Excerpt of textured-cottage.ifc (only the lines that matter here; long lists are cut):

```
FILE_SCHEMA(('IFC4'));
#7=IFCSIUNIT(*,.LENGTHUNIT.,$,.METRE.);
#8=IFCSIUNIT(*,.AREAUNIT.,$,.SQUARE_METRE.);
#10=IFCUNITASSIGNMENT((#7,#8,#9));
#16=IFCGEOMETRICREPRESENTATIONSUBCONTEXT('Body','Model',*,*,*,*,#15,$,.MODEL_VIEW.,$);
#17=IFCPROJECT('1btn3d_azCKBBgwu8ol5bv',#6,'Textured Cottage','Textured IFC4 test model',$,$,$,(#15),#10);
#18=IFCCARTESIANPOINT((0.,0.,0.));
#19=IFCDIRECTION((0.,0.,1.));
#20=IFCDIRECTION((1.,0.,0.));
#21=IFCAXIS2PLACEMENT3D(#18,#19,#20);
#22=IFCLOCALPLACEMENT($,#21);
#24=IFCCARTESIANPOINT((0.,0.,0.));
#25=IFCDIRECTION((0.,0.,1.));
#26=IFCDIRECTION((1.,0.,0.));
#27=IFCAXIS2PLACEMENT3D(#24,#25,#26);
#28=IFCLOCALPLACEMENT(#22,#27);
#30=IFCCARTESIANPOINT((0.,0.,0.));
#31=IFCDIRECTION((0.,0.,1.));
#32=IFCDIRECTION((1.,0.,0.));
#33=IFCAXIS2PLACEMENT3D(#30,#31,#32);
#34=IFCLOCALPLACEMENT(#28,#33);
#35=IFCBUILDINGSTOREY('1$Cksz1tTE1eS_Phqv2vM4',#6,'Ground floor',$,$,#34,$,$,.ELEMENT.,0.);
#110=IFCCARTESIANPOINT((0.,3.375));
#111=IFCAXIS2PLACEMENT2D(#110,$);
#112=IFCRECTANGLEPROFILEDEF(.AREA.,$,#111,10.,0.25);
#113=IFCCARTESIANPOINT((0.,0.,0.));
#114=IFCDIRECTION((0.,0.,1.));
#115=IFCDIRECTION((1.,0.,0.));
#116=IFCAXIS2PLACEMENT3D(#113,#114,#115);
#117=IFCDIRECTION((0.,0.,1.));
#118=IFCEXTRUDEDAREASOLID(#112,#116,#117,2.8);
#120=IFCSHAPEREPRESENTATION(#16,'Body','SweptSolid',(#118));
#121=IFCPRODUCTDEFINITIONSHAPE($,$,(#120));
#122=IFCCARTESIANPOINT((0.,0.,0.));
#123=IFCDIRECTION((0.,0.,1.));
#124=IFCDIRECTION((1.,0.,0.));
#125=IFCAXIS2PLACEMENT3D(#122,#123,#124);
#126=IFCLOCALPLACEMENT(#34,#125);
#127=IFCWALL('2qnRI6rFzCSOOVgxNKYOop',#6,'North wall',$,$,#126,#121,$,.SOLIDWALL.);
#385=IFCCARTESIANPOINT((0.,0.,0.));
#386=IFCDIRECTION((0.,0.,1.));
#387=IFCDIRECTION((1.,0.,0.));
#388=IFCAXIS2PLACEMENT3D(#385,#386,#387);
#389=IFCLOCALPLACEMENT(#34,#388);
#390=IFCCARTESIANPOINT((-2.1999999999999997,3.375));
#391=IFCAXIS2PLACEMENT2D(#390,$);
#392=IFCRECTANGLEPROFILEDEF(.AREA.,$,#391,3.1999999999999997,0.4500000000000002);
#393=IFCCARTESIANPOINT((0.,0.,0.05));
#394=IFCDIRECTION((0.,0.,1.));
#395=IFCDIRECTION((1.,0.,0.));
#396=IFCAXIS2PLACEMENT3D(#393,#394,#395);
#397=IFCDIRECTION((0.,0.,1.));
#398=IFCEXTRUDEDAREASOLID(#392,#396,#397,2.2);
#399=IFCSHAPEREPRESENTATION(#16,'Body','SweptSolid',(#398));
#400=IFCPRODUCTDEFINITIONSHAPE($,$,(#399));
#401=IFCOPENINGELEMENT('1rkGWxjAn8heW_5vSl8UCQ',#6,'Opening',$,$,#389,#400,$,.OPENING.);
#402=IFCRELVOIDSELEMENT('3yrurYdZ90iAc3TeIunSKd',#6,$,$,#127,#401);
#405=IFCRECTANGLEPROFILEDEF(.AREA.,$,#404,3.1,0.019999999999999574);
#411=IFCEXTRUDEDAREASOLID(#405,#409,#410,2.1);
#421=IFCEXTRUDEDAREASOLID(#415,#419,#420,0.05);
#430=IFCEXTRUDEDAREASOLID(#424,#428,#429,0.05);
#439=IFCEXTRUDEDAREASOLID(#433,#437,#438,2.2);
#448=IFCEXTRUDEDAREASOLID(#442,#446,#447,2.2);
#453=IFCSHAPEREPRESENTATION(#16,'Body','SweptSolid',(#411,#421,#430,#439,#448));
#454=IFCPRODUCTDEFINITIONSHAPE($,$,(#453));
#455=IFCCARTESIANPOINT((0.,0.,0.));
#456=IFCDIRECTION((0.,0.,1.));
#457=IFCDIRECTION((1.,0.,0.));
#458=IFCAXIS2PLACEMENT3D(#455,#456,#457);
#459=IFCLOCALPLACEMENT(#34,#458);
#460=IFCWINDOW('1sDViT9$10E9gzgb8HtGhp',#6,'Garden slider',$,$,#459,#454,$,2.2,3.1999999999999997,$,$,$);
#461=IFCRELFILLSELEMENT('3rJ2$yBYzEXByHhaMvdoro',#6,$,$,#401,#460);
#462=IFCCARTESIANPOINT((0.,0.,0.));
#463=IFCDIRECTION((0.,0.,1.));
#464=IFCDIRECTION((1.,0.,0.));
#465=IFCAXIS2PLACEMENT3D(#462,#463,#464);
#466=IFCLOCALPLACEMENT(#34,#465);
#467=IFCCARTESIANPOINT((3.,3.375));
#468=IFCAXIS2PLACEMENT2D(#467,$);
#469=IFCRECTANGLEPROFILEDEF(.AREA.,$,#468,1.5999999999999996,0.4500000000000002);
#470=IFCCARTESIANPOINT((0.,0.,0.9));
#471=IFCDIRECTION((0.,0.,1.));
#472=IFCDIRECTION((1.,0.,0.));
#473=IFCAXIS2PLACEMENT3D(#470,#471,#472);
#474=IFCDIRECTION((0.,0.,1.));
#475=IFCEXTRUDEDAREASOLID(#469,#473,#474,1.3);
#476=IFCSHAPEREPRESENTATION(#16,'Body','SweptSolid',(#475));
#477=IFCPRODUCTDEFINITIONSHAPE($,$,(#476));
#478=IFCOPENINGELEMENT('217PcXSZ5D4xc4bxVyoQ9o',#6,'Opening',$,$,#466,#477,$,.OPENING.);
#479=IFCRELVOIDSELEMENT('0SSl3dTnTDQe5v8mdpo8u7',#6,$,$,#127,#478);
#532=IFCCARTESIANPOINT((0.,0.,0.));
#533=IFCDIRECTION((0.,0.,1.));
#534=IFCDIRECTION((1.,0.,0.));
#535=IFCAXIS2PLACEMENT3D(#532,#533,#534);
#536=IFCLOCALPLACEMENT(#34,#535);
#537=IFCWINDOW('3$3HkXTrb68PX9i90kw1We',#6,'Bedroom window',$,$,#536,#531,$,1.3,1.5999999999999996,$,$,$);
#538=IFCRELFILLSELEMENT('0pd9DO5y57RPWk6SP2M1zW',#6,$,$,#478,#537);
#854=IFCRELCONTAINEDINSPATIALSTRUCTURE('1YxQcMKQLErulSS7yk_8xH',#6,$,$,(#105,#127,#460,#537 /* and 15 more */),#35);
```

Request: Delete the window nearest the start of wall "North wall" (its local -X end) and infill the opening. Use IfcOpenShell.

```python
import ifcopenshell
import ifcopenshell.api.feature
import ifcopenshell.api.root
import ifcopenshell.geom
import ifcopenshell.util.shape

model = ifcopenshell.open("textured-cottage.ifc")
settings = ifcopenshell.geom.settings()


def volume(element):
    """Net volume in cubic metres, openings subtracted."""
    shape = ifcopenshell.geom.create_shape(settings, element)
    return ifcopenshell.util.shape.get_volume(shape.geometry)


window = model.by_id(460)
opening = window.FillsVoids[0].RelatingOpeningElement
wall = opening.VoidsElements[0].RelatingBuildingElement
before = volume(wall)

ifcopenshell.api.root.remove_product(model, product=window)
ifcopenshell.api.feature.remove_feature(model, feature=opening)

after = volume(wall)

print(f"wall volume {before:.3f} -> {after:.3f} m3")

model.write("textured-cottage_updated.ifc")
```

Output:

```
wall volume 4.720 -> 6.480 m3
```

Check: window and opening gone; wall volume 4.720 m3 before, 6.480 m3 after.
